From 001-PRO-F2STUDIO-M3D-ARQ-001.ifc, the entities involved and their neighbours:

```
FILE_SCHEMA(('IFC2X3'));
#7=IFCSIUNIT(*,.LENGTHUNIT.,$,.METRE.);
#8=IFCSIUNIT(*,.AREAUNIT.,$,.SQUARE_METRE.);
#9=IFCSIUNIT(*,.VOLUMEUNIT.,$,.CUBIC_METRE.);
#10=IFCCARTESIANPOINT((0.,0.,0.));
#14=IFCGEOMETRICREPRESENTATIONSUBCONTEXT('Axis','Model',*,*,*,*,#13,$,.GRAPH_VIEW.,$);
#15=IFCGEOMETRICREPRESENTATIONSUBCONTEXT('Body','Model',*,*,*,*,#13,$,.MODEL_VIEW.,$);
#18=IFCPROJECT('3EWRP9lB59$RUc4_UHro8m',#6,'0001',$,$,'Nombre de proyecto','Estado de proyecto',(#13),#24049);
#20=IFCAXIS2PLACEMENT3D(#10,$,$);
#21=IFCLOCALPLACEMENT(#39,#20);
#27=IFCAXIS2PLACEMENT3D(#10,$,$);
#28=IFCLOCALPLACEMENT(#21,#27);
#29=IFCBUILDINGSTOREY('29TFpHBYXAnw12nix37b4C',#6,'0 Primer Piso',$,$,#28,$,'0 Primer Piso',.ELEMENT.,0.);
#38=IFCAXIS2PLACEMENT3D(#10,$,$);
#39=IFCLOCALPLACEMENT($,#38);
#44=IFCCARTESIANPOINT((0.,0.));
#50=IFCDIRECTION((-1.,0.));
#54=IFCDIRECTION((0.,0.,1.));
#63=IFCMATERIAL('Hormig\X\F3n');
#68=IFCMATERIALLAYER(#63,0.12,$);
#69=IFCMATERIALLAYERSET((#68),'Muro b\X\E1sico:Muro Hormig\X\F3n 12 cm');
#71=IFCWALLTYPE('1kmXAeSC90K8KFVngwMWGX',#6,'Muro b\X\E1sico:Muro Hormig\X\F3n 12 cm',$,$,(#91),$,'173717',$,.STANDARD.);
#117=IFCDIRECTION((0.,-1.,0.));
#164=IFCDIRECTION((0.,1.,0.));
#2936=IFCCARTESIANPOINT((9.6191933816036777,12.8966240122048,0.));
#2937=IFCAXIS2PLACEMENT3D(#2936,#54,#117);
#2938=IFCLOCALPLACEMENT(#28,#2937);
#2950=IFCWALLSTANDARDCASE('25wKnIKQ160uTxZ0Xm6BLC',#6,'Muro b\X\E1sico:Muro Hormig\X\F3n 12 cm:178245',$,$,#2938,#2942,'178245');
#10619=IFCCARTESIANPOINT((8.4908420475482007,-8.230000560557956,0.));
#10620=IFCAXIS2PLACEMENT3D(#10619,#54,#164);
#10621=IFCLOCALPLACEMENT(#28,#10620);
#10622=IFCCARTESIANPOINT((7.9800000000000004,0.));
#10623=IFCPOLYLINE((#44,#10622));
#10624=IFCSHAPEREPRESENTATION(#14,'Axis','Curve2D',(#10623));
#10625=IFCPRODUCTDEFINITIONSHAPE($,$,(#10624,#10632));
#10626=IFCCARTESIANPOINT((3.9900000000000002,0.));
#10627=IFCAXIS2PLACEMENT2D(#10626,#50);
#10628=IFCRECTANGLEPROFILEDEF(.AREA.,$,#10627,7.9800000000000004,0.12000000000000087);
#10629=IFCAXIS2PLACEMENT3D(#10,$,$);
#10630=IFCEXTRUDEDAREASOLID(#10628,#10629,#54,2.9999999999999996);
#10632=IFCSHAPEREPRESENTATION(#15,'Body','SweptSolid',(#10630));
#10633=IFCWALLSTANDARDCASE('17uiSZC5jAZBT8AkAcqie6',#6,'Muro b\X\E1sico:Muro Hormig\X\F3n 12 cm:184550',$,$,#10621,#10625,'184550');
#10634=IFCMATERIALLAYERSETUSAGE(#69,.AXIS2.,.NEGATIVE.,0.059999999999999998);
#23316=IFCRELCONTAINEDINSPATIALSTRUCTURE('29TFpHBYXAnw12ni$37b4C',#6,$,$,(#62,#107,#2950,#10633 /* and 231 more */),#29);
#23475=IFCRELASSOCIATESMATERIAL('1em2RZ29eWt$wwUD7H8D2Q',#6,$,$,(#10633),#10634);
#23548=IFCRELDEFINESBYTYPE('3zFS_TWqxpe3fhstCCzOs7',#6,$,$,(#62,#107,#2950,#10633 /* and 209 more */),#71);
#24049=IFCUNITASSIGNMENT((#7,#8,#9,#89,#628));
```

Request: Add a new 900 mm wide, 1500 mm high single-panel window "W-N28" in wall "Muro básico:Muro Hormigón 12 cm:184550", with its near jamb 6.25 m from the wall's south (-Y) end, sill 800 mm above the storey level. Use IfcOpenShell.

```python
import numpy as np
import ifcopenshell
import ifcopenshell.api.feature
import ifcopenshell.api.geometry
import ifcopenshell.api.root
import ifcopenshell.api.spatial
import ifcopenshell.api.type
import ifcopenshell.geom
import ifcopenshell.util.element
import ifcopenshell.util.placement
import ifcopenshell.util.representation
import ifcopenshell.util.shape
import ifcopenshell.util.unit

model = ifcopenshell.open("001-PRO-F2STUDIO-M3D-ARQ-001.ifc")
unit_scale = ifcopenshell.util.unit.calculate_unit_scale(model)
settings = ifcopenshell.geom.settings()


def volume(element):
    """Net volume in cubic metres, openings subtracted."""
    shape = ifcopenshell.geom.create_shape(settings, element)
    return ifcopenshell.util.shape.get_volume(shape.geometry)


wall = model.by_guid("17uiSZC5jAZBT8AkAcqie6")
storey = ifcopenshell.util.element.get_container(wall, ifc_class="IfcBuildingStorey")
context = ifcopenshell.util.representation.get_context(model, "Model", "Body", "MODEL_VIEW")
before = volume(wall)

width, height, from_end, sill = 0.9, 1.5, 6.25, 0.8  # metres

# The wall runs along its own X axis, and the end named is its -X end.
wall_shape = ifcopenshell.geom.create_shape(settings, wall)
x, y, z = ifcopenshell.util.shape.get_vertices(wall_shape.geometry).T
start = x.min() + from_end
face, thickness = float(y.min()), float(y.max() - y.min())
wall_matrix = ifcopenshell.util.placement.get_local_placement(wall.ObjectPlacement)
level = ifcopenshell.util.placement.get_local_placement(storey.ObjectPlacement)[2, 3]


def in_wall(x, y):
    """Placement at x, y metres in the wall's axes, at sill height."""
    matrix = wall_matrix.copy()
    matrix[:, 3] = wall_matrix @ np.array([x / unit_scale, y / unit_scale, 0.0, 1.0])
    matrix[2, 3] = level + sill / unit_scale
    return matrix


# Opening: a box that overshoots both wall faces by 50 mm.
opening = ifcopenshell.api.root.create_entity(model, ifc_class="IfcOpeningElement")
box = ifcopenshell.api.geometry.add_wall_representation(
    model, context=context, length=width, height=height, thickness=thickness + 0.1
)
ifcopenshell.api.geometry.assign_representation(model, product=opening, representation=box)
ifcopenshell.api.geometry.edit_object_placement(model, product=opening, matrix=in_wall(start, face - 0.05), is_si=False)
ifcopenshell.api.feature.add_feature(model, feature=opening, element=wall)

window = ifcopenshell.api.root.create_entity(model, ifc_class="IfcWindow", name="W-N28")
window.OverallWidth, window.OverallHeight = width / unit_scale, height / unit_scale
body = ifcopenshell.api.geometry.add_window_representation(
    model,
    context=context,
    overall_width=window.OverallWidth,
    overall_height=window.OverallHeight,
    partition_type="SINGLE_PANEL",
)
ifcopenshell.api.geometry.assign_representation(model, product=window, representation=body)
ifcopenshell.api.spatial.assign_container(model, products=[window], relating_structure=storey)
fills = ifcopenshell.api.feature.add_filling(model, opening=opening, element=window)
fills.OwnerHistory = window.OwnerHistory  # required in IFC2X3

# IFC2X3 keeps the operation on the window style.
style = ifcopenshell.api.root.create_entity(model, ifc_class="IfcWindowStyle", name="W-N28")
style.OperationType, style.ConstructionType = "SINGLE_PANEL", "NOTDEFINED"
style.ParameterTakesPrecedence = style.Sizeable = False
ifcopenshell.api.type.assign_type(model, related_objects=[window], relating_type=style)

# Centre the window in the wall's thickness.
ifcopenshell.api.geometry.edit_object_placement(model, product=window, matrix=in_wall(start, face), is_si=False)
window_shape = ifcopenshell.geom.create_shape(settings, window)
depth = ifcopenshell.util.shape.get_vertices(window_shape.geometry)[:, 1]
offset = face + thickness / 2 - (depth.min() + depth.max()) / 2
ifcopenshell.api.geometry.edit_object_placement(model, product=window, matrix=in_wall(start, offset), is_si=False)

after = volume(wall)

print(f"wall volume {before:.3f} -> {after:.3f} m3")

model.write("001-PRO-F2STUDIO-M3D-ARQ-001-out.ifc")
```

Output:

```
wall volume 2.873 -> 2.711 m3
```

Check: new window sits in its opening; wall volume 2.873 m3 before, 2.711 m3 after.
